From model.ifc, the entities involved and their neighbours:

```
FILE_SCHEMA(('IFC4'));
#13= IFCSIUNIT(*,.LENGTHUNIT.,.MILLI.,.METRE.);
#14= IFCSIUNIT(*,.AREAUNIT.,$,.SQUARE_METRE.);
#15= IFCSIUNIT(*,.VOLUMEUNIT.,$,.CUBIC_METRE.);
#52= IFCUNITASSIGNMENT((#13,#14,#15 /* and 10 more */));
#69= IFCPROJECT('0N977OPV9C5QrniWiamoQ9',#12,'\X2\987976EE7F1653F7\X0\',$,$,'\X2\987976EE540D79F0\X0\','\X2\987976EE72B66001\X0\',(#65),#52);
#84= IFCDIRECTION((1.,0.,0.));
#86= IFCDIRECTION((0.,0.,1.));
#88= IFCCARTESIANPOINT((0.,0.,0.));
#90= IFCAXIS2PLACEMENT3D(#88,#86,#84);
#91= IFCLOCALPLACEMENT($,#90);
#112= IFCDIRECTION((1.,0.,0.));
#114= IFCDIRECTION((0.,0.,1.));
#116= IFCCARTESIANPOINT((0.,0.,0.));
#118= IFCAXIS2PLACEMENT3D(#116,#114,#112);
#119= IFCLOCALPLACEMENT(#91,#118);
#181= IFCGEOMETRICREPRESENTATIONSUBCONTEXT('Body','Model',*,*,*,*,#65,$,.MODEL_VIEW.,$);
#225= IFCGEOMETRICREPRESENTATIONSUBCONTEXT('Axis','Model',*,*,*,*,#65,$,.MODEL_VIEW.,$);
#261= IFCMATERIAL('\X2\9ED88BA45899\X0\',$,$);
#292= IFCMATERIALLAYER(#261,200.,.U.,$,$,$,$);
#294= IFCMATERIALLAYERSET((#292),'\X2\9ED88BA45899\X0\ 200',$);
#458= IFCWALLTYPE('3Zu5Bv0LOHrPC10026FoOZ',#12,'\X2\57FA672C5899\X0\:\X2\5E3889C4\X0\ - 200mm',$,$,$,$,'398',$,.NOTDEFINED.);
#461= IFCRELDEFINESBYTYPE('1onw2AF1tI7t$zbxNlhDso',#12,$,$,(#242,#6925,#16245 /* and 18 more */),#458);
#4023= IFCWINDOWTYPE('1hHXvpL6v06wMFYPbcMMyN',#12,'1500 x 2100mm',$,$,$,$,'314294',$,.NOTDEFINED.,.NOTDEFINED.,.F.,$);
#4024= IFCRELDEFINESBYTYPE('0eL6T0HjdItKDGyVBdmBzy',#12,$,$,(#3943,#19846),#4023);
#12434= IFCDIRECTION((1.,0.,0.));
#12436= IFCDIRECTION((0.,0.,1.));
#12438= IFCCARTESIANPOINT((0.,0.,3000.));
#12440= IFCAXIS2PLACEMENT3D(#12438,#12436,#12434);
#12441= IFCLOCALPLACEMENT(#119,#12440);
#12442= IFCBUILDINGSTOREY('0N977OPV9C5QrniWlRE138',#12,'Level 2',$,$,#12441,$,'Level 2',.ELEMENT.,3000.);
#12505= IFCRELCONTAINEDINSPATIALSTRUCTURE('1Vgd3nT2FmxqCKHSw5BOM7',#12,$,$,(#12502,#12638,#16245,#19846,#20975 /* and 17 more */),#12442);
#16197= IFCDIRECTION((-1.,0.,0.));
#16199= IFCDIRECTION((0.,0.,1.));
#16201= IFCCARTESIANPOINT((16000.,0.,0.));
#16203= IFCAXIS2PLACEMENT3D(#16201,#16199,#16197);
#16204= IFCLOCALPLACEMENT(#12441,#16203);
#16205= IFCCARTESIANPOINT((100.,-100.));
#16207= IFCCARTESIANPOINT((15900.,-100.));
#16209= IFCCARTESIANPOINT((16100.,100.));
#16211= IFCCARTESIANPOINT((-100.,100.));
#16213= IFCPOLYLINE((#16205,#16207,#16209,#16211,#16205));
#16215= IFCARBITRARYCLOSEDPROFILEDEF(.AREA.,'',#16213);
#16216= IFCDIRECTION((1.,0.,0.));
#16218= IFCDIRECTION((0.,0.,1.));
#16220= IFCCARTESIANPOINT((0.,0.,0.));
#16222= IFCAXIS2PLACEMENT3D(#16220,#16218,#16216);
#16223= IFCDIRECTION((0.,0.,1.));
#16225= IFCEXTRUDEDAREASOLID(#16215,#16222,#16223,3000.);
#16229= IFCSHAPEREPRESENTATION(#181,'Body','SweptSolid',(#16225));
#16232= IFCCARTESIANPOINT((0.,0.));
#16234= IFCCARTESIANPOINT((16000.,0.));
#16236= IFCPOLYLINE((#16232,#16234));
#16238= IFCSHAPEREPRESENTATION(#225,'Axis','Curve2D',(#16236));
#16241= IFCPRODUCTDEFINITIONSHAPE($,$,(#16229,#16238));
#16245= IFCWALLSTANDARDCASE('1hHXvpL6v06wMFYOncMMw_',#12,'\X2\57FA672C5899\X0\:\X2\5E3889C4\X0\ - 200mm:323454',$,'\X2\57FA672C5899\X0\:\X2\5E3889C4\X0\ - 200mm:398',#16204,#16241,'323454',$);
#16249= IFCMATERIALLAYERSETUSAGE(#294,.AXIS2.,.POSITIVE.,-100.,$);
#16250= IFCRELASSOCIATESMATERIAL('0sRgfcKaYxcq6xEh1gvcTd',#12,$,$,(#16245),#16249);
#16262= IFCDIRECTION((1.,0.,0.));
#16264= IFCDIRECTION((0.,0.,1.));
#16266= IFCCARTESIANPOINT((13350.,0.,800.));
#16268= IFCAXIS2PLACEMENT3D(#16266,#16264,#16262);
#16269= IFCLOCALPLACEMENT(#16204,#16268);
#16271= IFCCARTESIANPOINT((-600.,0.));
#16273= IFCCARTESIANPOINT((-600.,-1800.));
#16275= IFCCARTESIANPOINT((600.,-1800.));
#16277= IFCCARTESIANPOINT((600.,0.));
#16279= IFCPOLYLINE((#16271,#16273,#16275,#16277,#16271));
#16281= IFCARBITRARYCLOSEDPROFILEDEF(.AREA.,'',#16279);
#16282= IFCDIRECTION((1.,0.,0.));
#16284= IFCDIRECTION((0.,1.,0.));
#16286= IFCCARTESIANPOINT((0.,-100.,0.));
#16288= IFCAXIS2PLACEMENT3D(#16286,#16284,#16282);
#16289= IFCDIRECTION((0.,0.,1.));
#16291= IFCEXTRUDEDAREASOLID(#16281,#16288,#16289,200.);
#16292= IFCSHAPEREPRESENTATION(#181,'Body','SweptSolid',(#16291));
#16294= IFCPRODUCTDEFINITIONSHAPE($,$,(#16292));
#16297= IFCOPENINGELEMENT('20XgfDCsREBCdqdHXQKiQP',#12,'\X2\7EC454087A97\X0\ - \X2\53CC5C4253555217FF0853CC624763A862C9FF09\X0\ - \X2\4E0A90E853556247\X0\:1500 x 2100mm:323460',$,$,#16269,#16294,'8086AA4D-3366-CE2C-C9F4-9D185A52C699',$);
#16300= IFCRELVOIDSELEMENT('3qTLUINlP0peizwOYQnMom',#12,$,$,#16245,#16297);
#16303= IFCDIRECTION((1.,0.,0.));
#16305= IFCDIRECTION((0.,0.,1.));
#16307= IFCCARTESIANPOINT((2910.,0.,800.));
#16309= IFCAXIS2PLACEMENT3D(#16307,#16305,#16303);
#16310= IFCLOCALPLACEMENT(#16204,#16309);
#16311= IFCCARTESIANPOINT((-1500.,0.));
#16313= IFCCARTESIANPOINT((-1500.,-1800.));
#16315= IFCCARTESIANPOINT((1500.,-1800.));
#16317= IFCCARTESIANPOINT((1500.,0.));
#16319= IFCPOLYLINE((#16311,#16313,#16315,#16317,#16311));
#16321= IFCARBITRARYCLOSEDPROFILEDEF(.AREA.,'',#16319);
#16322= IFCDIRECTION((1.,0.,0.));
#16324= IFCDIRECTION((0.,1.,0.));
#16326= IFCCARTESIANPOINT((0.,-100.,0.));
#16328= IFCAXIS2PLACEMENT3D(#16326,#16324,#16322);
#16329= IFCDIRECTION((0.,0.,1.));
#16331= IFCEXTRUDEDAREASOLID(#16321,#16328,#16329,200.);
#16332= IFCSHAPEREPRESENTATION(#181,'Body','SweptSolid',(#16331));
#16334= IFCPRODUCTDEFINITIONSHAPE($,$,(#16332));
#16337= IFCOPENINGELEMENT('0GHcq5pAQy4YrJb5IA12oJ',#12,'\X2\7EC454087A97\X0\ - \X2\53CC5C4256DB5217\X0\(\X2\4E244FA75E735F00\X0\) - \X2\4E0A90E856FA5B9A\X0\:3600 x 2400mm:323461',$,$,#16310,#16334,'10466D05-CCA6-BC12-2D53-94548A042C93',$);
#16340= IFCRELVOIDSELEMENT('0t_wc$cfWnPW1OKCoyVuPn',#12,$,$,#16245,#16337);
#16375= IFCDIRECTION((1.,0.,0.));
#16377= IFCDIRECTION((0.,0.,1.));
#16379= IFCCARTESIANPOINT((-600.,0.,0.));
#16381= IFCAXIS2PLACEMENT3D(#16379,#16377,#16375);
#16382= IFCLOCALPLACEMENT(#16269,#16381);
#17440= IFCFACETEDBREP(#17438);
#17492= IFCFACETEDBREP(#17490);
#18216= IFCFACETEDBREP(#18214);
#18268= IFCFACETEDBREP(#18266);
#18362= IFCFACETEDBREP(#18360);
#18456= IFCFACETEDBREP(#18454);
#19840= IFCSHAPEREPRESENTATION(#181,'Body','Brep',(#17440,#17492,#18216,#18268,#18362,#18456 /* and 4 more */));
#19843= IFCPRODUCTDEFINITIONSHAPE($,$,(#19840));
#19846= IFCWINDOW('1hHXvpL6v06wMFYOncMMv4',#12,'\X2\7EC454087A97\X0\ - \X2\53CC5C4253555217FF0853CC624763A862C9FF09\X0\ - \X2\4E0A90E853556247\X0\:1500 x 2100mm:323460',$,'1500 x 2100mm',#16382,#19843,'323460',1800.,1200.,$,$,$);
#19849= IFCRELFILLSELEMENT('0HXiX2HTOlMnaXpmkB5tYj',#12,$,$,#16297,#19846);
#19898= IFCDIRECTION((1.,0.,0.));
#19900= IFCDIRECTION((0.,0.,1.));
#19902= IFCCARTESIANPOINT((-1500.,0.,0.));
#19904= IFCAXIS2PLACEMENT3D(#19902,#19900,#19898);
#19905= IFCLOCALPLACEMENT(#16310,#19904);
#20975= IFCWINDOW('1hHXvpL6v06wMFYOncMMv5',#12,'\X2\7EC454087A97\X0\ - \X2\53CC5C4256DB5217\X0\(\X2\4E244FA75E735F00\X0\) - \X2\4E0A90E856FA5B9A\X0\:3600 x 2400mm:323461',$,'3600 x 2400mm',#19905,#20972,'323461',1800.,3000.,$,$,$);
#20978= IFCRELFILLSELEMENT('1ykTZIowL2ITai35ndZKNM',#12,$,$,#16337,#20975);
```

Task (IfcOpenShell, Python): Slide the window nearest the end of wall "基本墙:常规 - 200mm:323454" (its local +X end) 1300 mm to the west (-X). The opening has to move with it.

```python
import ifcopenshell
import ifcopenshell.api.geometry
import ifcopenshell.util.placement

model = ifcopenshell.open("model.ifc")

window = model.by_guid("1hHXvpL6v06wMFYOncMMv4")
opening = window.FillsVoids[0].RelatingOpeningElement
wall = opening.VoidsElements[0].RelatingBuildingElement

wall_matrix = ifcopenshell.util.placement.get_local_placement(wall.ObjectPlacement)
shift = wall_matrix[:3, 0] * 1300.0
before = ifcopenshell.util.placement.get_local_placement(window.ObjectPlacement)[:3, 3].copy()

# The window is placed relative to its opening, so it follows when the opening moves.
matrix = ifcopenshell.util.placement.get_local_placement(opening.ObjectPlacement)
matrix[:3, 3] += shift
ifcopenshell.api.geometry.edit_object_placement(
    model, product=opening, matrix=matrix, is_si=False, should_transform_children=True
)

after = ifcopenshell.util.placement.get_local_placement(window.ObjectPlacement)[:3, 3]
print("window moved by", (after - before).round(3) + 0.0)

model.write("model_updated.ifc")
```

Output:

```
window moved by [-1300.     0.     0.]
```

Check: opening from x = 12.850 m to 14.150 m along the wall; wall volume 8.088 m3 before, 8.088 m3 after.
